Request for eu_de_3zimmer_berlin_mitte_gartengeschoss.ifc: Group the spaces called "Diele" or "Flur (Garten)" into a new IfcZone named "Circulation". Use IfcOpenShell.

First a look at what the model holds.

```python
import ifcopenshell

model = ifcopenshell.open("eu_de_3zimmer_berlin_mitte_gartengeschoss.ifc")
print(model.schema)
seen = {}
for space in model.by_type("IfcSpace"):
    seen[space.LongName] = seen.get(space.LongName, 0) + 1
for name, count in sorted(seen.items(), key=str):
    print(count, "x", name)
print("zones:", [z.Name for z in model.by_type("IfcZone")][:20])
```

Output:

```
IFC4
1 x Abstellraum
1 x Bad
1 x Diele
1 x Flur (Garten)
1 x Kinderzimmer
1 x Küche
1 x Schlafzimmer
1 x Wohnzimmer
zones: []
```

```python
import ifcopenshell
import ifcopenshell.api.group
import ifcopenshell.api.root

model = ifcopenshell.open("eu_de_3zimmer_berlin_mitte_gartengeschoss.ifc")

names = {"Diele", "Flur (Garten)"}
spaces = [s for s in model.by_type("IfcSpace") if s.LongName in names]

zone = ifcopenshell.api.root.create_entity(model, ifc_class="IfcZone", name="Circulation")
ifcopenshell.api.group.assign_group(model, products=spaces, group=zone)
print(len(spaces), "spaces in", zone.Name)

model.write("eu_de_3zimmer_berlin_mitte_gartengeschoss-out.ifc")
```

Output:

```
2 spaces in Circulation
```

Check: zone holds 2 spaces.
